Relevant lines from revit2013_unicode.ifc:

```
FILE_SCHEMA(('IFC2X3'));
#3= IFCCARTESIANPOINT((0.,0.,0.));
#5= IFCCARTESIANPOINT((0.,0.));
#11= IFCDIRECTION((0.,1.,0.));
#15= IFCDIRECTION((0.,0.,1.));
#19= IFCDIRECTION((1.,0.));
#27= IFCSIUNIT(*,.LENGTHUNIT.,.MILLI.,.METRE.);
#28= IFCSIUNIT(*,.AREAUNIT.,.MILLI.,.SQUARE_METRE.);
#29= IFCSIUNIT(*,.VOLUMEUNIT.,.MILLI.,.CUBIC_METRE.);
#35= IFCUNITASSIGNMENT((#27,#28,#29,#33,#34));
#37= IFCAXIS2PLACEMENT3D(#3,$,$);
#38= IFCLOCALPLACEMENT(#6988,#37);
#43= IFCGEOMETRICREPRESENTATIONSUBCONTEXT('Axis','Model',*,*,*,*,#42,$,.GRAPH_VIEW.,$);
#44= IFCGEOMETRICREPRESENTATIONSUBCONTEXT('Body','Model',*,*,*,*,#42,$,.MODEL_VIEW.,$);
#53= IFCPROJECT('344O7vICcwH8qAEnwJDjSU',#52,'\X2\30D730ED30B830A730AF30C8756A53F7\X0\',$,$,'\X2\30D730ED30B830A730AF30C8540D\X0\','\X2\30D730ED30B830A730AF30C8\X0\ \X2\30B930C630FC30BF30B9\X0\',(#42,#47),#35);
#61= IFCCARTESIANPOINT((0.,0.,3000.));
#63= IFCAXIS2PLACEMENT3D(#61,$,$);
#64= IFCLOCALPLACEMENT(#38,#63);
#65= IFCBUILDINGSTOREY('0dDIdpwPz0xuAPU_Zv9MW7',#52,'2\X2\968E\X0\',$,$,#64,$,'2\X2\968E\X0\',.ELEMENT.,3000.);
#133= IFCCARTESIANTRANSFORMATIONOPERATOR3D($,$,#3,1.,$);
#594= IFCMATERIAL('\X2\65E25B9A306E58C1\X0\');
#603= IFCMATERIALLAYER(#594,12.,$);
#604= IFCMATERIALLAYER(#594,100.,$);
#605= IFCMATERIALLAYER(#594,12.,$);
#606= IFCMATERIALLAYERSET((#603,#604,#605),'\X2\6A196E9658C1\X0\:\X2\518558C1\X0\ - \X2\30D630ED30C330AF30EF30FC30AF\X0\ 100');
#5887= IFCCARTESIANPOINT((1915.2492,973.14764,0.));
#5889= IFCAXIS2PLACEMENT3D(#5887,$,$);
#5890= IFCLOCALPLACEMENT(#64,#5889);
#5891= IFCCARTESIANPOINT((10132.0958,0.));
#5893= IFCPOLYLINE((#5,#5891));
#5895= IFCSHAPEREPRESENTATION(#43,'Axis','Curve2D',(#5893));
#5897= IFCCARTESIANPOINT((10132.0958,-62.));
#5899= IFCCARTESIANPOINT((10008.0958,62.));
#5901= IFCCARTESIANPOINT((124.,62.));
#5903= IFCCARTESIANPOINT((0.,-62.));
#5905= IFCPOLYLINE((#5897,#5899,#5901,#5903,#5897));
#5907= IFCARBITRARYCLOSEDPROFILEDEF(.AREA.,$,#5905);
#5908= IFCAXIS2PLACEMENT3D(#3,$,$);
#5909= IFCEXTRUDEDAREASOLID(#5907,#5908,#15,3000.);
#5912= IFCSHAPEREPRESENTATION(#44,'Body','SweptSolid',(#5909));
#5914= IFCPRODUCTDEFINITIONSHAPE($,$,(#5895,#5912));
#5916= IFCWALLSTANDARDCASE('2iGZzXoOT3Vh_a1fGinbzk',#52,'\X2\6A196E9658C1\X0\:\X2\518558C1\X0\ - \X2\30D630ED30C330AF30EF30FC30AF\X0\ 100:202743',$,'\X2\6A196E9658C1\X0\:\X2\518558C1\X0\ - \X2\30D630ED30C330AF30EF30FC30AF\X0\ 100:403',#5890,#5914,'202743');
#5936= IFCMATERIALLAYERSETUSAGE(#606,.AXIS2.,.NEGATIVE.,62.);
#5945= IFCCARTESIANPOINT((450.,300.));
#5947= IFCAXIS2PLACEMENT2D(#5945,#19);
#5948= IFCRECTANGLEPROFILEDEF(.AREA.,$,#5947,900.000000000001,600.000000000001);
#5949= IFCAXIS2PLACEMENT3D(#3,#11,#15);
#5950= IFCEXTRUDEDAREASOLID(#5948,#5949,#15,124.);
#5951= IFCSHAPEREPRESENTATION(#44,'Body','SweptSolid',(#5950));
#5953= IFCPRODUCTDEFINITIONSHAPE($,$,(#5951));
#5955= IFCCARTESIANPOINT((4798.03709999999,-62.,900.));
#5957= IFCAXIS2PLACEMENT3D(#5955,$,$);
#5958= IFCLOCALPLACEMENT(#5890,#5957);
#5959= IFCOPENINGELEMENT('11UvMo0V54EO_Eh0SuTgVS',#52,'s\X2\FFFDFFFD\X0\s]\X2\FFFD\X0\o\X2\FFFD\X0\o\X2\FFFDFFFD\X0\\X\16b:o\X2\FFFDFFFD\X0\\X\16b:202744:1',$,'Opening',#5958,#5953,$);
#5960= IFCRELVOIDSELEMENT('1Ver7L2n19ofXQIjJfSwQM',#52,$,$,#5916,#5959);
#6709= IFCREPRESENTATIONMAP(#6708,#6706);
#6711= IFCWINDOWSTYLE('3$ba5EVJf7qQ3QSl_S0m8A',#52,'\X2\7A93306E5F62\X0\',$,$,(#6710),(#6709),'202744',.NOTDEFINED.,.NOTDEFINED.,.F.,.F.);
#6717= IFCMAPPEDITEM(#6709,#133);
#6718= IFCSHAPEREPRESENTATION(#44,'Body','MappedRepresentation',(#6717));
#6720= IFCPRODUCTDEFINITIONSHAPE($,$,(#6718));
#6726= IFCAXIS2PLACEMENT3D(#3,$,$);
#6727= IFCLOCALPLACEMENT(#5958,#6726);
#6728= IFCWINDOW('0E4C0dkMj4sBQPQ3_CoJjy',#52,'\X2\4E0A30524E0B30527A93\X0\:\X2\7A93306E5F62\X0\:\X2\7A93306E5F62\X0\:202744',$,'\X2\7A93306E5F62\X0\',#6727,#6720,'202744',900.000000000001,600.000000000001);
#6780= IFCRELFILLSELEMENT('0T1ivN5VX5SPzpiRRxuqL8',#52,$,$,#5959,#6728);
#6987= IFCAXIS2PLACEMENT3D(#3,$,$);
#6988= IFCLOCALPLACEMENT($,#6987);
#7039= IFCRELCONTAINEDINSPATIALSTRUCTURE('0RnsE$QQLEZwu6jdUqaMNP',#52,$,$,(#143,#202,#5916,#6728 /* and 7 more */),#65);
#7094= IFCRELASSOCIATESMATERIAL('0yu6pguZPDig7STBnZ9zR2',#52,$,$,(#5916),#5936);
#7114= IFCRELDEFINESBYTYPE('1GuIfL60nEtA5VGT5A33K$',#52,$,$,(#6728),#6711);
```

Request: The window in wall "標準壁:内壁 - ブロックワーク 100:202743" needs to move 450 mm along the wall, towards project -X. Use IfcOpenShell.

```python
import ifcopenshell
import ifcopenshell.api.geometry
import ifcopenshell.util.placement
import ifcopenshell.util.unit

model = ifcopenshell.open("revit2013_unicode.ifc")
unit_scale = ifcopenshell.util.unit.calculate_unit_scale(model)

window = model.by_guid("0E4C0dkMj4sBQPQ3_CoJjy")
opening = window.FillsVoids[0].RelatingOpeningElement
wall = opening.VoidsElements[0].RelatingBuildingElement

wall_matrix = ifcopenshell.util.placement.get_local_placement(wall.ObjectPlacement)
shift = wall_matrix[:3, 0] * -0.45 / unit_scale
before = ifcopenshell.util.placement.get_local_placement(window.ObjectPlacement)[:3, 3].copy()

# The window is placed relative to its opening, so it follows when the opening moves.
matrix = ifcopenshell.util.placement.get_local_placement(opening.ObjectPlacement)
matrix[:3, 3] += shift
ifcopenshell.api.geometry.edit_object_placement(
    model, product=opening, matrix=matrix, is_si=False, should_transform_children=True
)

after = ifcopenshell.util.placement.get_local_placement(window.ObjectPlacement)[:3, 3]
print("window moved by", (after - before).round(3) + 0.0)

model.write("revit2013_unicode_updated.ifc")
```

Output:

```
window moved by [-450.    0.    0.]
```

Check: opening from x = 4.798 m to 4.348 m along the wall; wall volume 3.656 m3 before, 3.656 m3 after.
